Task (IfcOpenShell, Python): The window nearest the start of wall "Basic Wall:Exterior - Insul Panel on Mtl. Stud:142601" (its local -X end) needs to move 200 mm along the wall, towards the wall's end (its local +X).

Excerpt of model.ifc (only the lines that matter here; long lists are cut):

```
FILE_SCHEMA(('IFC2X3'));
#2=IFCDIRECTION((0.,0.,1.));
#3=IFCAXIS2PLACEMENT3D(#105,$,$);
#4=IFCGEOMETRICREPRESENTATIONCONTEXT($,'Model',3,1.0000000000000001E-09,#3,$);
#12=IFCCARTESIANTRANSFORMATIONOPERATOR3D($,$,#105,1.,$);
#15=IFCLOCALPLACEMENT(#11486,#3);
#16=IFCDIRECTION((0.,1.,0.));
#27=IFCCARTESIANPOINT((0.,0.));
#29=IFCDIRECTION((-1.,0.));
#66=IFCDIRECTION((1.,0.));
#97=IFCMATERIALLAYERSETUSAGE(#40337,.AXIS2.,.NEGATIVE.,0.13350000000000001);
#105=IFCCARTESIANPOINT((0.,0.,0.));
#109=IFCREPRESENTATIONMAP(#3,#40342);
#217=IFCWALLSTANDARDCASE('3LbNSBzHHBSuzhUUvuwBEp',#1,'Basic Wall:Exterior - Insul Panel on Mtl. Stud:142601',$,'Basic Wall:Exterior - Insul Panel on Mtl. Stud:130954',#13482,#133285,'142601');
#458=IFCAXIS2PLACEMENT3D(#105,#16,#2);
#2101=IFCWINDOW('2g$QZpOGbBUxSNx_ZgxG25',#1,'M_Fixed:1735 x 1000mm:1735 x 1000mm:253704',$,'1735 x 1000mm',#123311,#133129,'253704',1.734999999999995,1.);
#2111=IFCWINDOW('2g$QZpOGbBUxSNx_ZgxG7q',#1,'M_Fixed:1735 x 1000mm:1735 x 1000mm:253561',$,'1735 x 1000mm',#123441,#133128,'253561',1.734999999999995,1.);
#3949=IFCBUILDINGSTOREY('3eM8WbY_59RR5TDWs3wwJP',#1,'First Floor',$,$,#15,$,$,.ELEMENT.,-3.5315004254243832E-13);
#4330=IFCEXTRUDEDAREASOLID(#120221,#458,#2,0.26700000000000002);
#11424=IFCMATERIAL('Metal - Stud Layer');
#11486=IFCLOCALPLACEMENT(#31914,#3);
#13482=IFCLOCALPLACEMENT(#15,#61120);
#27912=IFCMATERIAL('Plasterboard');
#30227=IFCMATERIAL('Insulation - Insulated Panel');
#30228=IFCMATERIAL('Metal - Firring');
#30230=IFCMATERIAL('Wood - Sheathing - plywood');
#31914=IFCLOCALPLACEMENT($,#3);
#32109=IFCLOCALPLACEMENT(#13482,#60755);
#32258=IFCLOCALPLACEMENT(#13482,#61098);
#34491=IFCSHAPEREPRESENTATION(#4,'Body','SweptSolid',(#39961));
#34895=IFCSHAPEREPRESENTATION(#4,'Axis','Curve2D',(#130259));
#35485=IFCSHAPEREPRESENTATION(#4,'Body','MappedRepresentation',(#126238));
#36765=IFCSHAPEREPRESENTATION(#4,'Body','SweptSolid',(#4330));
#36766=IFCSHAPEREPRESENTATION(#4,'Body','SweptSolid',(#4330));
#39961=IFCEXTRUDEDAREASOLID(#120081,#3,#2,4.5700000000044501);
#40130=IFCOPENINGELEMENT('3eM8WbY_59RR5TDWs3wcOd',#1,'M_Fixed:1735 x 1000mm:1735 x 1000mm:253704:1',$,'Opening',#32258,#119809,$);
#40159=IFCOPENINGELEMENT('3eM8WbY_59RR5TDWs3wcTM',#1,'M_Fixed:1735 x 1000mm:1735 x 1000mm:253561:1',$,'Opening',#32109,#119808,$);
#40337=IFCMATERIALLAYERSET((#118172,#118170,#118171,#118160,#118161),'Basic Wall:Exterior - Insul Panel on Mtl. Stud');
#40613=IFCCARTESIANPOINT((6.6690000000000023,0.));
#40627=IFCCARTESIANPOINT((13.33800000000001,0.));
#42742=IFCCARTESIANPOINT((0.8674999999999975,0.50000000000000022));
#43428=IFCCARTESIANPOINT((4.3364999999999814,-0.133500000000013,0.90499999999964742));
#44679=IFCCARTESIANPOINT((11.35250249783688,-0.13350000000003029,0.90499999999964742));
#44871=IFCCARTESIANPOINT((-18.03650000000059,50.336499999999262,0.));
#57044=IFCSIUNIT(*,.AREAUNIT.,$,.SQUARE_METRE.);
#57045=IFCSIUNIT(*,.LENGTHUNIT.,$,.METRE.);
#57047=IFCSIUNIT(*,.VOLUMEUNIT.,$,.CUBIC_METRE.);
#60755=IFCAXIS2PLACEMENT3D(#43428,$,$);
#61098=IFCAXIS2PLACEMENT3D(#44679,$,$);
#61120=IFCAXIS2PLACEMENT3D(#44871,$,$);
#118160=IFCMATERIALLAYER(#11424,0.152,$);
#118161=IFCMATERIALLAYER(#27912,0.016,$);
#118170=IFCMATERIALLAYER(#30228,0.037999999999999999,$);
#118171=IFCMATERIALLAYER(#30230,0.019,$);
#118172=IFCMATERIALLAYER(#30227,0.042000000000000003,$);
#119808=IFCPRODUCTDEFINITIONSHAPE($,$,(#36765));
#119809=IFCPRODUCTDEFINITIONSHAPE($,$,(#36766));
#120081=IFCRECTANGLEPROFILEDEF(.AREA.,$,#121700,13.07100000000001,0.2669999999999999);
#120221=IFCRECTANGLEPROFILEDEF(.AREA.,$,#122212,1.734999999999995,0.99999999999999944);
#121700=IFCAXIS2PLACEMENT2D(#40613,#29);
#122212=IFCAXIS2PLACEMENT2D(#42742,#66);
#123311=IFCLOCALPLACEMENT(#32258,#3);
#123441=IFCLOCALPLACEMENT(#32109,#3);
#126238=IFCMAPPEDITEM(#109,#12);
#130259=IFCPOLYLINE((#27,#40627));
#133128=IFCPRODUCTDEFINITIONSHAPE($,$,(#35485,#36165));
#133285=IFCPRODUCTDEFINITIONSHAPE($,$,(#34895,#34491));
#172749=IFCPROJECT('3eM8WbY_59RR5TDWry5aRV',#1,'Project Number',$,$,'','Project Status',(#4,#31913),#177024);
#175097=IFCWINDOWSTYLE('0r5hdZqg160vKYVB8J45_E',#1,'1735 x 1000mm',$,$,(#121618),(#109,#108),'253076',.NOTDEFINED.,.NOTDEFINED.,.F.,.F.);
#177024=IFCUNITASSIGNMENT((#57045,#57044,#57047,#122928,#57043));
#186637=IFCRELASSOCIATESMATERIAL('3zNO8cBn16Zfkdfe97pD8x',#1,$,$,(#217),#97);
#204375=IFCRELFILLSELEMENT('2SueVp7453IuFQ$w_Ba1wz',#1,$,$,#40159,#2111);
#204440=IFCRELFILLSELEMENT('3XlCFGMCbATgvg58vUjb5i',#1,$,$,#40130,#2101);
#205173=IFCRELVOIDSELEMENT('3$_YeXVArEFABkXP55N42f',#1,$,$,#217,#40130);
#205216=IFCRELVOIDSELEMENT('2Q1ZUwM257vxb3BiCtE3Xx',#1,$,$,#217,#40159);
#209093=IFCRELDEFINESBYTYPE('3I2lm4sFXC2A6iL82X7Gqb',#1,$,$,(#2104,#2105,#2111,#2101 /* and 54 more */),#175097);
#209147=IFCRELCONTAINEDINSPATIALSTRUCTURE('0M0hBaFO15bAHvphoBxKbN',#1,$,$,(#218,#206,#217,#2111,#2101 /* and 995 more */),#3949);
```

```python
import ifcopenshell
import ifcopenshell.api.geometry
import ifcopenshell.util.placement

model = ifcopenshell.open("model.ifc")

window = model.by_id(2111)
opening = window.FillsVoids[0].RelatingOpeningElement
wall = opening.VoidsElements[0].RelatingBuildingElement

wall_matrix = ifcopenshell.util.placement.get_local_placement(wall.ObjectPlacement)
shift = wall_matrix[:3, 0] * 0.2
before = ifcopenshell.util.placement.get_local_placement(window.ObjectPlacement)[:3, 3].copy()

# The window is placed relative to its opening, so it follows when the opening moves.
matrix = ifcopenshell.util.placement.get_local_placement(opening.ObjectPlacement)
matrix[:3, 3] += shift
ifcopenshell.api.geometry.edit_object_placement(
    model, product=opening, matrix=matrix, is_si=False, should_transform_children=True
)

after = ifcopenshell.util.placement.get_local_placement(window.ObjectPlacement)[:3, 3]
print("window moved by", (after - before).round(3) + 0.0)

model.write("model_rev.ifc")
```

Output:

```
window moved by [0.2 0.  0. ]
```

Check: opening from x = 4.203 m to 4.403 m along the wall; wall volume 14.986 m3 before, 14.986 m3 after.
